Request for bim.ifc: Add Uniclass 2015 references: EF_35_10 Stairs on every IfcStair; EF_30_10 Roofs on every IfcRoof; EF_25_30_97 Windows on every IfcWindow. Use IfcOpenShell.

First a look at what the model holds.

```python
import ifcopenshell

model = ifcopenshell.open("bim.ifc")
print(model.schema)
print("classifications:", [c.Name for c in model.by_type("IfcClassification")])
for ifc_class in ("IfcDoor", "IfcRoof", "IfcStair", "IfcWall", "IfcWindow"):
    print(ifc_class, len(model.by_type(ifc_class)))
```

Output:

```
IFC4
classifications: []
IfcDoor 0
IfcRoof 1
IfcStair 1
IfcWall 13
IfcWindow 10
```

```python
import ifcopenshell
import ifcopenshell.api.classification

model = ifcopenshell.open("bim.ifc")

system = ifcopenshell.api.classification.add_classification(model, classification="Uniclass 2015")

codes = {
    "IfcStair": ("EF_35_10", "Stairs"),
    "IfcRoof": ("EF_30_10", "Roofs"),
    "IfcWindow": ("EF_25_30_97", "Windows"),
}
for ifc_class, (code, name) in codes.items():
    products = model.by_type(ifc_class)
    ifcopenshell.api.classification.add_reference(
        model, products=products, classification=system, identification=code, name=name
    )
    print(code, len(products))

model.write("bim_v2.ifc")
```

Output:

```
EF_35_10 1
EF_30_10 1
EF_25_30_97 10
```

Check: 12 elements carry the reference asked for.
